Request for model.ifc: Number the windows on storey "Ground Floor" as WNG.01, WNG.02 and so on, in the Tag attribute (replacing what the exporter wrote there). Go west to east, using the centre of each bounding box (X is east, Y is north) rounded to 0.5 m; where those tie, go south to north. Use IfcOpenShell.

First a look at what the model holds.

```python
import ifcopenshell
import ifcopenshell.util.element
import ifcopenshell.util.placement

model = ifcopenshell.open("model.ifc")
print(model.schema)
storey = next(s for s in model.by_type("IfcBuildingStorey") if s.Name == "Ground Floor")
windows = [e for e in ifcopenshell.util.element.get_decomposition(storey) if e.is_a("IfcWindow")]
for e in sorted(windows, key=lambda e: e.id()):
    origin = ifcopenshell.util.placement.get_local_placement(e.ObjectPlacement)[:3, 3]
    print(e.id(), e.Tag, e.Name, origin.round(2) + 0.0, sep=" | ")
```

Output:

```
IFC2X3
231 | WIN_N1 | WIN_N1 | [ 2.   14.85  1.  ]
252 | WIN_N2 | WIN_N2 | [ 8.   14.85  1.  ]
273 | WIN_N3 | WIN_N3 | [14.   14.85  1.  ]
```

```python
import ifcopenshell
import ifcopenshell.geom
import ifcopenshell.util.element
import ifcopenshell.util.shape

model = ifcopenshell.open("model.ifc")
settings = ifcopenshell.geom.settings()
settings.set("use-world-coords", True)


def centre(element):
    shape = ifcopenshell.geom.create_shape(settings, element)
    return ifcopenshell.util.shape.get_bbox_centroid(shape.geometry)


storey = next(s for s in model.by_type("IfcBuildingStorey") if s.Name == "Ground Floor")
windows = [e for e in ifcopenshell.util.element.get_decomposition(storey) if e.is_a("IfcWindow")]

# Insertion points can sit at a corner or the storey origin, so sort by the geometry (in metres).
centres = {e: centre(e) for e in windows}
windows.sort(key=lambda e: (round(centres[e][0] / 0.5), centres[e][1]))

for i, e in enumerate(windows, start=1):
    number = f"WNG.{i:02d}"
    e.Tag = number
    print(e.id(), number)

model.write("model_edited.ifc")
```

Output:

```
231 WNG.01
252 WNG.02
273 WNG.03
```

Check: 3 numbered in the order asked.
